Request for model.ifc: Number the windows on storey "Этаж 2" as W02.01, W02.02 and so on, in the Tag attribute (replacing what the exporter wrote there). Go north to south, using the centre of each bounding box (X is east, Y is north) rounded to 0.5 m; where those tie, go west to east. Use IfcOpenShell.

First a look at what the model holds.

```python
import ifcopenshell
import ifcopenshell.util.element
import ifcopenshell.util.placement

model = ifcopenshell.open("model.ifc")
print(model.schema)
storey = next(s for s in model.by_type("IfcBuildingStorey") if s.Name == "Этаж 2")
windows = [e for e in ifcopenshell.util.element.get_decomposition(storey) if e.is_a("IfcWindow")]
for e in sorted(windows, key=lambda e: e.id()):
    origin = ifcopenshell.util.placement.get_local_placement(e.ObjectPlacement)[:3, 3]
    print(e.id(), e.Tag, e.Name, origin.round(2) + 0.0, sep=" | ")
```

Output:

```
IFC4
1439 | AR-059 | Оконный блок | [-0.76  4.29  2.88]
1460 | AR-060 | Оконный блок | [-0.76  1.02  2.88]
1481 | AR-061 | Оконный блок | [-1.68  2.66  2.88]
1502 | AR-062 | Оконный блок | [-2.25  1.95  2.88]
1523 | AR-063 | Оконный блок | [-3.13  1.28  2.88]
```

```python
import ifcopenshell
import ifcopenshell.geom
import ifcopenshell.util.element
import ifcopenshell.util.shape

model = ifcopenshell.open("model.ifc")
settings = ifcopenshell.geom.settings()
settings.set("use-world-coords", True)


def centre(element):
    shape = ifcopenshell.geom.create_shape(settings, element)
    return ifcopenshell.util.shape.get_bbox_centroid(shape.geometry)


storey = next(s for s in model.by_type("IfcBuildingStorey") if s.Name == "Этаж 2")
windows = [e for e in ifcopenshell.util.element.get_decomposition(storey) if e.is_a("IfcWindow")]

# Insertion points can sit at a corner or the storey origin, so sort by the geometry (in metres).
centres = {e: centre(e) for e in windows}
windows.sort(key=lambda e: (-round(centres[e][1] / 0.5), centres[e][0]))

for i, e in enumerate(windows, start=1):
    number = f"W02.{i:02d}"
    e.Tag = number
    print(e.id(), number)

model.write("model-out.ifc")
```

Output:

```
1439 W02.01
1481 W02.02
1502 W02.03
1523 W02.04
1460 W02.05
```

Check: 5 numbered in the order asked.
